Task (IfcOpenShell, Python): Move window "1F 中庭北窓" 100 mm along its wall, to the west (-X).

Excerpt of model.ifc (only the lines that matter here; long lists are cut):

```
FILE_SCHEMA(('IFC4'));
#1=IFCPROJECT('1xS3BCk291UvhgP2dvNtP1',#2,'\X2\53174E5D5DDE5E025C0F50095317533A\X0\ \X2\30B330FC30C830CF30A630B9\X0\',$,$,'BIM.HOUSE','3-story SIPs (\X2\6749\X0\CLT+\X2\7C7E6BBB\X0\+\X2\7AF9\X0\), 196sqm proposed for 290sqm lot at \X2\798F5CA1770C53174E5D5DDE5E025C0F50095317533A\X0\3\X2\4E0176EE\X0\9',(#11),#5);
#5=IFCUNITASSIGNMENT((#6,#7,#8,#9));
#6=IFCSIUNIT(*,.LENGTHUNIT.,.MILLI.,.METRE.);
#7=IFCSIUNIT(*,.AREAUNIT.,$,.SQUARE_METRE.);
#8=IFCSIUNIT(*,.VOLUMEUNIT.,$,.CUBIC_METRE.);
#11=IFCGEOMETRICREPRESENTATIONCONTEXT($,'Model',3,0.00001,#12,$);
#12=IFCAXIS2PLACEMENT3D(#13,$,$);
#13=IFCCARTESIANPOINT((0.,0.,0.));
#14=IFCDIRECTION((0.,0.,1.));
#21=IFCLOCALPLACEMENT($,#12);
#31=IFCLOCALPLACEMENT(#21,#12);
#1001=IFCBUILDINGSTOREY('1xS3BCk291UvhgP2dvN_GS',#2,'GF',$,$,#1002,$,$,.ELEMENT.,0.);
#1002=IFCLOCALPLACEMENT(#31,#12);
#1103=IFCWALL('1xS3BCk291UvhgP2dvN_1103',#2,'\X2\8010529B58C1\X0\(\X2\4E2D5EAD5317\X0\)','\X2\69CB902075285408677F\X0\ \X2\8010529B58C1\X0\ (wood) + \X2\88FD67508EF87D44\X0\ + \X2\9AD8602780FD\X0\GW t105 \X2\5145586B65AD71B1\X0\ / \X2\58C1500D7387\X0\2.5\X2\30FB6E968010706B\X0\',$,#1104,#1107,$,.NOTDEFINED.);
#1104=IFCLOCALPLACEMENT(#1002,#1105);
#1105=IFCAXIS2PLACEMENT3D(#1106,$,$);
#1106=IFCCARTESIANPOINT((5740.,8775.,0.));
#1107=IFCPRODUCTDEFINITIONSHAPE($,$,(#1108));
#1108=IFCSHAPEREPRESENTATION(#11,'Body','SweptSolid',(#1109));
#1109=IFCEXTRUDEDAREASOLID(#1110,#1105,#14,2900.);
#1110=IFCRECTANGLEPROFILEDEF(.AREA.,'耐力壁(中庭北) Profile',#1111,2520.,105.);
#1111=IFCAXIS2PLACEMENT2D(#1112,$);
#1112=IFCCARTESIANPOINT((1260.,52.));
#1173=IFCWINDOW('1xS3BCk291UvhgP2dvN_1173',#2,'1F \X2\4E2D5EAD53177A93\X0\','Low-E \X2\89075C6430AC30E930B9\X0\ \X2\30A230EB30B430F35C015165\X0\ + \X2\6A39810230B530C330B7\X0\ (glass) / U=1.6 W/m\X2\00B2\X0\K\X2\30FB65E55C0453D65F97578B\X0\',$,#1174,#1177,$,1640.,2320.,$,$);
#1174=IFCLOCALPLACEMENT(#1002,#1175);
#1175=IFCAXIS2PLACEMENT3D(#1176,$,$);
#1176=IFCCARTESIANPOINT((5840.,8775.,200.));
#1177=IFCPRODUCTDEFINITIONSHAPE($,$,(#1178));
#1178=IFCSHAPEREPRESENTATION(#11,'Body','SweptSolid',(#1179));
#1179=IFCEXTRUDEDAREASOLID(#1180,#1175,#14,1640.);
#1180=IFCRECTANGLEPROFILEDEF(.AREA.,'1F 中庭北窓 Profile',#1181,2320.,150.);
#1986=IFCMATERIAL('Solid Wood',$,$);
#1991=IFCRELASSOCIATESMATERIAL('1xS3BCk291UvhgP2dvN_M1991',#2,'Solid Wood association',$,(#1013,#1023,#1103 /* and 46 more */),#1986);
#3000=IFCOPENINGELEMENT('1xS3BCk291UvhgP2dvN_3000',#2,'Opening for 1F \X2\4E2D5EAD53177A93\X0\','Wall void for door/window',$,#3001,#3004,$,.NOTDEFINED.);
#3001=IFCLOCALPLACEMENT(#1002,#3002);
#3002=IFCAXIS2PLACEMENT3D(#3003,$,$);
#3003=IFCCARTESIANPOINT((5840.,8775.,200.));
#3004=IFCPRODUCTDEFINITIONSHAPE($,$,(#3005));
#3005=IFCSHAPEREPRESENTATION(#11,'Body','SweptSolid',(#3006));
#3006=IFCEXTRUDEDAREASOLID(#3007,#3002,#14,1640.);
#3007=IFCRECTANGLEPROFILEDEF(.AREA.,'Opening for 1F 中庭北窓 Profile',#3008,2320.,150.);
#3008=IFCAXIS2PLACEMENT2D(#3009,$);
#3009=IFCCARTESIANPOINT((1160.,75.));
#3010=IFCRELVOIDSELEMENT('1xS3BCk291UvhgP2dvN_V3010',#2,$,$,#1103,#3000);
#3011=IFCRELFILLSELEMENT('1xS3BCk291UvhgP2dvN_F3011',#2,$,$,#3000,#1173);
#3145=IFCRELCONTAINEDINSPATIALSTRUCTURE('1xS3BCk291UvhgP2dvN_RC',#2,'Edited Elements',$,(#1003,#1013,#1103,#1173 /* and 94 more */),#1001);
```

```python
import ifcopenshell
import ifcopenshell.api.geometry
import ifcopenshell.util.placement
import ifcopenshell.util.unit

model = ifcopenshell.open("model.ifc")
unit_scale = ifcopenshell.util.unit.calculate_unit_scale(model)

window = model.by_id(1173)
opening = window.FillsVoids[0].RelatingOpeningElement
wall = opening.VoidsElements[0].RelatingBuildingElement

wall_matrix = ifcopenshell.util.placement.get_local_placement(wall.ObjectPlacement)
shift = wall_matrix[:3, 0] * -0.1 / unit_scale
before = ifcopenshell.util.placement.get_local_placement(window.ObjectPlacement)[:3, 3].copy()

# The window is not placed relative to its opening, so move both.
for product in (opening, window):
    matrix = ifcopenshell.util.placement.get_local_placement(product.ObjectPlacement)
    matrix[:3, 3] += shift
    ifcopenshell.api.geometry.edit_object_placement(model, product=product, matrix=matrix, is_si=False)

after = ifcopenshell.util.placement.get_local_placement(window.ObjectPlacement)[:3, 3]
print("window moved by", (after - before).round(3) + 0.0)

model.write("model_edited.ifc")
```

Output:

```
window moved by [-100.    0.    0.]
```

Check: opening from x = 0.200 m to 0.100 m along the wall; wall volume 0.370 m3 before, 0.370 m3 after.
